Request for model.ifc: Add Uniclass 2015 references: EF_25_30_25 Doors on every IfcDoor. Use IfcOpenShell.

First a look at what the model holds.

```python
import ifcopenshell

model = ifcopenshell.open("model.ifc")
print(model.schema)
print("classifications:", [c.Name for c in model.by_type("IfcClassification")])
for ifc_class in ("IfcDoor", "IfcRoof", "IfcStair", "IfcWall", "IfcWindow"):
    print(ifc_class, len(model.by_type(ifc_class)))
```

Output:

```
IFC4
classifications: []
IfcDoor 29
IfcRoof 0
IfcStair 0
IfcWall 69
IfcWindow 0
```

```python
import ifcopenshell
import ifcopenshell.api.classification

model = ifcopenshell.open("model.ifc")

system = ifcopenshell.api.classification.add_classification(model, classification="Uniclass 2015")

codes = {
    "IfcDoor": ("EF_25_30_25", "Doors"),
}
for ifc_class, (code, name) in codes.items():
    products = model.by_type(ifc_class)
    ifcopenshell.api.classification.add_reference(
        model, products=products, classification=system, identification=code, name=name
    )
    print(code, len(products))

model.write("model-out.ifc")
```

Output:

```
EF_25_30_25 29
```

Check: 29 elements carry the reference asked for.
